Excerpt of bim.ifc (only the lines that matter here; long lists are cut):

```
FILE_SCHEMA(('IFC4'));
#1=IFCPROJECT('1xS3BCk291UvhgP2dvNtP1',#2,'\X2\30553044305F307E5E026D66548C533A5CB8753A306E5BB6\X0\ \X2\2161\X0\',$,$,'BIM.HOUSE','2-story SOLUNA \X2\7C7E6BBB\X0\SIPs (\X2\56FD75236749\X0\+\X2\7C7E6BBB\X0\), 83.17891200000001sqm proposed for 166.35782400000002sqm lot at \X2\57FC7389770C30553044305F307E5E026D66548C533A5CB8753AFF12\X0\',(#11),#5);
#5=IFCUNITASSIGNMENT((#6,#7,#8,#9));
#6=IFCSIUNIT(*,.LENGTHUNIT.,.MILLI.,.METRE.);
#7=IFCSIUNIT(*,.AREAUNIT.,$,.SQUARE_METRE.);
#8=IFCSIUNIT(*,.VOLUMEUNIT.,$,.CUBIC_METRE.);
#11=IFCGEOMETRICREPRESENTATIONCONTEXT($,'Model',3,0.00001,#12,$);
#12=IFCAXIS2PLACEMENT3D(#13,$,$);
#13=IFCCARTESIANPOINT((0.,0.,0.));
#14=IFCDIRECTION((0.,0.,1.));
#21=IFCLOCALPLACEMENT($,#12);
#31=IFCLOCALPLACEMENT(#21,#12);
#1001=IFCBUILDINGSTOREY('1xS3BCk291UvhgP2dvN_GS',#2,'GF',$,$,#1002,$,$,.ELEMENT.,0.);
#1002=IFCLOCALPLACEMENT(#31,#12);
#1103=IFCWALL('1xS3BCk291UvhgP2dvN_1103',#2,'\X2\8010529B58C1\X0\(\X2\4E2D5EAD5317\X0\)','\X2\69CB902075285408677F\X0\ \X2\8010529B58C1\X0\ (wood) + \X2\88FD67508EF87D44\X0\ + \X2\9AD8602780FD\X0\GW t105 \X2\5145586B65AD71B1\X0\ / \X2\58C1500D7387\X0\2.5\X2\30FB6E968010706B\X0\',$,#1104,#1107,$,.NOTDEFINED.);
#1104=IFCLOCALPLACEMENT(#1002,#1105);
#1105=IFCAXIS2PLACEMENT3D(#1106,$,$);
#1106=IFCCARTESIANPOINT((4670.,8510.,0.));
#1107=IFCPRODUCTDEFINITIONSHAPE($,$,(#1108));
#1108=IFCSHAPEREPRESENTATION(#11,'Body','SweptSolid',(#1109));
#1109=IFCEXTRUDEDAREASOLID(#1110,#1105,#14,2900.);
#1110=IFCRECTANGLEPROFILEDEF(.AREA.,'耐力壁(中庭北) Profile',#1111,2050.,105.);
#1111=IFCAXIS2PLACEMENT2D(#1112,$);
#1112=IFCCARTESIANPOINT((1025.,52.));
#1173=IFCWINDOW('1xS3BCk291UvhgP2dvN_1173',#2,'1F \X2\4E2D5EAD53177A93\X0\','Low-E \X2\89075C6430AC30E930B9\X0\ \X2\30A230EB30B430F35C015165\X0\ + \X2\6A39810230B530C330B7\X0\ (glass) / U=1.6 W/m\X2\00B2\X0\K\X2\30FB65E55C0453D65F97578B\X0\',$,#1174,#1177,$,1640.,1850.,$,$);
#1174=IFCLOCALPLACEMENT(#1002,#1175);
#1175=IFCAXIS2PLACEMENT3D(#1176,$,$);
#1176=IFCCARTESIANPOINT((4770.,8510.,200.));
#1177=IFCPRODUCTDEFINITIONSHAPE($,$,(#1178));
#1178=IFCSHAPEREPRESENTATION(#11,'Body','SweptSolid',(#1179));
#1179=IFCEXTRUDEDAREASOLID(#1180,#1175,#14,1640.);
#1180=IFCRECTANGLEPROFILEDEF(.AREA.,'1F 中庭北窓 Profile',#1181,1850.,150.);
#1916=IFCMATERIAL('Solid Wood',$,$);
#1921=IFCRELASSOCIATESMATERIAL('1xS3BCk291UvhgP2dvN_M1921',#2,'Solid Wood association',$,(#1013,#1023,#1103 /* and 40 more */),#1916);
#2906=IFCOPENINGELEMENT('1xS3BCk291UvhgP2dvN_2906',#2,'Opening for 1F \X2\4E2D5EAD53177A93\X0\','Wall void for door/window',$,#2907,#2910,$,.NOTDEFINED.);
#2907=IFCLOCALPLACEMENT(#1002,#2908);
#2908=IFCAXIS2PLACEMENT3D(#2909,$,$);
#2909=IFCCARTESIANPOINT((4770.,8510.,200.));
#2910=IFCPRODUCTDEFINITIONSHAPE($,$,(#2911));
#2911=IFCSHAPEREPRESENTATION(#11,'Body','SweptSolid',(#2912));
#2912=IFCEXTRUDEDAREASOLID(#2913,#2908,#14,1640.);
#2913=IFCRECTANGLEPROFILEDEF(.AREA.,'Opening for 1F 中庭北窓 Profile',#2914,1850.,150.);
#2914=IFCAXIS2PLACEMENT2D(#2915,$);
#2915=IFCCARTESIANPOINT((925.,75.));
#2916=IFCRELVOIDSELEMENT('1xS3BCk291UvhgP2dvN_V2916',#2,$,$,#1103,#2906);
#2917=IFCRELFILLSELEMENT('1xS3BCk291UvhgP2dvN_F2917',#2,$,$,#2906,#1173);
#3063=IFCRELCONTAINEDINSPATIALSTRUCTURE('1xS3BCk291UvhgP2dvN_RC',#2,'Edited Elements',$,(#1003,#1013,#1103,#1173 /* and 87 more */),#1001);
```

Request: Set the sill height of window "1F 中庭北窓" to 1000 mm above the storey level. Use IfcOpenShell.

```python
import numpy as np
import ifcopenshell
import ifcopenshell.api.geometry
import ifcopenshell.geom
import ifcopenshell.util.element
import ifcopenshell.util.placement
import ifcopenshell.util.shape
import ifcopenshell.util.unit

model = ifcopenshell.open("bim.ifc")
unit_scale = ifcopenshell.util.unit.calculate_unit_scale(model)

window = model.by_id(1173)
opening = window.FillsVoids[0].RelatingOpeningElement
storey = ifcopenshell.util.element.get_container(window, ifc_class="IfcBuildingStorey")
level = ifcopenshell.util.placement.get_local_placement(storey.ObjectPlacement)[2, 3]

# The opening's origin need not be at the sill, so measure its lowest point.
shape = ifcopenshell.geom.create_shape(ifcopenshell.geom.settings(), opening)
bottom = ifcopenshell.util.shape.get_shape_bottom_elevation(shape, shape.geometry) / unit_scale
dz = level + 1 / unit_scale - bottom

shift = np.array([0.0, 0.0, dz])
# The window is not placed relative to its opening, so move both.
for product in (opening, window):
    matrix = ifcopenshell.util.placement.get_local_placement(product.ObjectPlacement)
    matrix[:3, 3] += shift
    ifcopenshell.api.geometry.edit_object_placement(model, product=product, matrix=matrix, is_si=False)

print(f"moved by {dz * unit_scale:+.3f} m")

model.write("bim_updated.ifc")
```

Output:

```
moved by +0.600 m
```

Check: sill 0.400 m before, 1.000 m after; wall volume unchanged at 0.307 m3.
